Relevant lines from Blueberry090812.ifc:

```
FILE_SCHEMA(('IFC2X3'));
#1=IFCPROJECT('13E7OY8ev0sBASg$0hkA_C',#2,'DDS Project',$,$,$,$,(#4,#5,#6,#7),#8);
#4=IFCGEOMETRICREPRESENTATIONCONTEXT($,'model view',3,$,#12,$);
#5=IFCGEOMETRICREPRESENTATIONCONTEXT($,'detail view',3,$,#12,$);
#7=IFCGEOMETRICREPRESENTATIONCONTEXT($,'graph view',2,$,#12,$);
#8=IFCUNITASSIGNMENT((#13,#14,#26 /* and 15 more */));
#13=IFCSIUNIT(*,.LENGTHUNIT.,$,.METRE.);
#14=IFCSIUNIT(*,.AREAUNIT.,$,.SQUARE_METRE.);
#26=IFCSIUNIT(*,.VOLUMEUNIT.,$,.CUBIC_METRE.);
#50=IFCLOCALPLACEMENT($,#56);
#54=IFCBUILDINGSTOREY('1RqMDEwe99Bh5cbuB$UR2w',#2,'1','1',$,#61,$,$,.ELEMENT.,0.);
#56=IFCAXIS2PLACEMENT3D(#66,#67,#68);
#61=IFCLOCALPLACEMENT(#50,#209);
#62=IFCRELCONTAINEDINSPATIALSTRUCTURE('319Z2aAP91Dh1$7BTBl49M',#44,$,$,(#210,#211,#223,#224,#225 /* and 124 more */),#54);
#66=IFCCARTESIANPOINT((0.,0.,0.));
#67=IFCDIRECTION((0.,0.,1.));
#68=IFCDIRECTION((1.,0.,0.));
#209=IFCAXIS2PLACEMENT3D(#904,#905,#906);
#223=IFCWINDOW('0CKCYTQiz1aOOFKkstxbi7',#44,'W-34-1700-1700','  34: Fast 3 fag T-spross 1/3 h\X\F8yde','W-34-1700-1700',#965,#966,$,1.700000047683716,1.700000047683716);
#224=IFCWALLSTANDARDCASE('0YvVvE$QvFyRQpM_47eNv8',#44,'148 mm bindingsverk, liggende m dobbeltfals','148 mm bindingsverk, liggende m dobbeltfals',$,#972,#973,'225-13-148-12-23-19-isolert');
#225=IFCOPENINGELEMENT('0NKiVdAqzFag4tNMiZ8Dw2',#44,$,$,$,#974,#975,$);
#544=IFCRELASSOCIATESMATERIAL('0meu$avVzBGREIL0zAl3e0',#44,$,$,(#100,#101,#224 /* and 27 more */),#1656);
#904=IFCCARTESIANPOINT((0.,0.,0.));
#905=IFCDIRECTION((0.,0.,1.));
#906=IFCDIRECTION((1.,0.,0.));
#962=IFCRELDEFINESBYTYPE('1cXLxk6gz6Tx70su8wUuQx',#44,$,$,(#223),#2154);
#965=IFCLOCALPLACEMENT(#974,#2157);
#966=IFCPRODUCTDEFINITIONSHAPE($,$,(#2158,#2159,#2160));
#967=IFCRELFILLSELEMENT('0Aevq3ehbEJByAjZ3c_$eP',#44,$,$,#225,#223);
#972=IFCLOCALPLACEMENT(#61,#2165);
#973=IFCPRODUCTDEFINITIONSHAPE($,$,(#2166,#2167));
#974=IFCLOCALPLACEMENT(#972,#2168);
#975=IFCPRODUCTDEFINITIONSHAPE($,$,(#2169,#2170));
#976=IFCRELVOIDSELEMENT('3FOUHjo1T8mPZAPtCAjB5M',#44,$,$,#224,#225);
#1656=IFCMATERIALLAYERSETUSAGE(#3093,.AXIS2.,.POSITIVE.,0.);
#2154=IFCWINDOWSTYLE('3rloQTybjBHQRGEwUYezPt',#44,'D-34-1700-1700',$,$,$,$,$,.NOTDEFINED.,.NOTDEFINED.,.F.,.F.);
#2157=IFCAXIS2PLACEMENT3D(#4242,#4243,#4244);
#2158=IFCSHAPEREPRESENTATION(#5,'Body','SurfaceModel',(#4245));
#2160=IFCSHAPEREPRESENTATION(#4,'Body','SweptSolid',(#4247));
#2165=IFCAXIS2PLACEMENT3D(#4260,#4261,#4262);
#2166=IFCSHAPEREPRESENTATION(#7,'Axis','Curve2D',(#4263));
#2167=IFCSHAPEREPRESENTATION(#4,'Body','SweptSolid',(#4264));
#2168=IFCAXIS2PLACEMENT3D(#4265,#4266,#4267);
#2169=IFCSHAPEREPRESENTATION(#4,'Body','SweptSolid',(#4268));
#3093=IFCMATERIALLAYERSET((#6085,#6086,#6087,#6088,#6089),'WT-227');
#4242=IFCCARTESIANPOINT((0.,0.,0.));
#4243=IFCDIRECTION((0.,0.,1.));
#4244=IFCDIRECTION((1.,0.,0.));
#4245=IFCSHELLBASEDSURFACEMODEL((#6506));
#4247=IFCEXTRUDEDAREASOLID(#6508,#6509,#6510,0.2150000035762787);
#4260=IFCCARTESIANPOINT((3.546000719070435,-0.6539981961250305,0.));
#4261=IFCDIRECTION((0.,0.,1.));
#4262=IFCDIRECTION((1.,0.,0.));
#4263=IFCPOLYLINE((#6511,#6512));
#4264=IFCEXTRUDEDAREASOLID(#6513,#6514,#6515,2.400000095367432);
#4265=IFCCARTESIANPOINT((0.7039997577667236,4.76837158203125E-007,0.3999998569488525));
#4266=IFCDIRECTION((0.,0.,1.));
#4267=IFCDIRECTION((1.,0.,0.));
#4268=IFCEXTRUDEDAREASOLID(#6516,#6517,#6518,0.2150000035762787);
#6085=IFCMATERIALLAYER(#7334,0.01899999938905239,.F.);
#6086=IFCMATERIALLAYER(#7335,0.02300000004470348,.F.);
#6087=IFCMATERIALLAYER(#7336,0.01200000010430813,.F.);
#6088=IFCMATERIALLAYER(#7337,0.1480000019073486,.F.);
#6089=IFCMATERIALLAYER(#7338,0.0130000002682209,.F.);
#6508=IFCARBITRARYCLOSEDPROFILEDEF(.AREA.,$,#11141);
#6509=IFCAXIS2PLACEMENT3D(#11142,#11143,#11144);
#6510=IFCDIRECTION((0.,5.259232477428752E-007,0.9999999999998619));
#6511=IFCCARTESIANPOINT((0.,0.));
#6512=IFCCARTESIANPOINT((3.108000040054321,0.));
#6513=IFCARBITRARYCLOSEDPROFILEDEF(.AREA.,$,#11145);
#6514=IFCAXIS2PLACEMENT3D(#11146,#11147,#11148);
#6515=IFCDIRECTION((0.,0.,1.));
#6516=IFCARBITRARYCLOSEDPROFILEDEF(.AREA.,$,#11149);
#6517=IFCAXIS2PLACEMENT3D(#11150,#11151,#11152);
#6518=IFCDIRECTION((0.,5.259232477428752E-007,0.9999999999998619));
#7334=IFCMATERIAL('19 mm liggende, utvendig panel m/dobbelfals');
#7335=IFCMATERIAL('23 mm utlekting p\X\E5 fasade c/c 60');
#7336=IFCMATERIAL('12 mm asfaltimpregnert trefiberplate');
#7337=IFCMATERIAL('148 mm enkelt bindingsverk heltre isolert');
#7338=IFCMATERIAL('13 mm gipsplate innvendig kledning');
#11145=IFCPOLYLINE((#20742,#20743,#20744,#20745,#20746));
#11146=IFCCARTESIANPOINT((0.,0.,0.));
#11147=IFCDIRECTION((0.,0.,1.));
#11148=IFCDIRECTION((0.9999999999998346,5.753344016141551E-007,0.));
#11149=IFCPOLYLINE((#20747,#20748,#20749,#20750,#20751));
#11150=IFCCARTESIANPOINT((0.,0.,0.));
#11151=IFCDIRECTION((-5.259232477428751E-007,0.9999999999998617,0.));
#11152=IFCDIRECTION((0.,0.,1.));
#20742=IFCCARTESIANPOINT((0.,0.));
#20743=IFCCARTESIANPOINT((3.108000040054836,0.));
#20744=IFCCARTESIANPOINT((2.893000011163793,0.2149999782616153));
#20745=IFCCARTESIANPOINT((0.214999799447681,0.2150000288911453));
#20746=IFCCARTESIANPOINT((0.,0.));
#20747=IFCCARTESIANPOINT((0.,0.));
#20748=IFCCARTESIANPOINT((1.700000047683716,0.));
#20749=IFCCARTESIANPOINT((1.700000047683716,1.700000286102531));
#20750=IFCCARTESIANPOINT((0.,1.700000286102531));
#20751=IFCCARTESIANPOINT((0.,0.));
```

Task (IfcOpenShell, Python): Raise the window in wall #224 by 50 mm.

```python
import numpy as np
import ifcopenshell
import ifcopenshell.api.geometry
import ifcopenshell.util.placement
import ifcopenshell.util.unit

model = ifcopenshell.open("Blueberry090812.ifc")
unit_scale = ifcopenshell.util.unit.calculate_unit_scale(model)

window = model.by_guid("0CKCYTQiz1aOOFKkstxbi7")
opening = window.FillsVoids[0].RelatingOpeningElement
dz = 0.05 / unit_scale

shift = np.array([0.0, 0.0, dz])
# The window is placed relative to its opening, so it follows when the opening moves.
matrix = ifcopenshell.util.placement.get_local_placement(opening.ObjectPlacement)
matrix[:3, 3] += shift
ifcopenshell.api.geometry.edit_object_placement(
    model, product=opening, matrix=matrix, is_si=False, should_transform_children=True
)

print(f"moved by {dz * unit_scale:+.3f} m")

model.write("Blueberry090812_v2.ifc")
```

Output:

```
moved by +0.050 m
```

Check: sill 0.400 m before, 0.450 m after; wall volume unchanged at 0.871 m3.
